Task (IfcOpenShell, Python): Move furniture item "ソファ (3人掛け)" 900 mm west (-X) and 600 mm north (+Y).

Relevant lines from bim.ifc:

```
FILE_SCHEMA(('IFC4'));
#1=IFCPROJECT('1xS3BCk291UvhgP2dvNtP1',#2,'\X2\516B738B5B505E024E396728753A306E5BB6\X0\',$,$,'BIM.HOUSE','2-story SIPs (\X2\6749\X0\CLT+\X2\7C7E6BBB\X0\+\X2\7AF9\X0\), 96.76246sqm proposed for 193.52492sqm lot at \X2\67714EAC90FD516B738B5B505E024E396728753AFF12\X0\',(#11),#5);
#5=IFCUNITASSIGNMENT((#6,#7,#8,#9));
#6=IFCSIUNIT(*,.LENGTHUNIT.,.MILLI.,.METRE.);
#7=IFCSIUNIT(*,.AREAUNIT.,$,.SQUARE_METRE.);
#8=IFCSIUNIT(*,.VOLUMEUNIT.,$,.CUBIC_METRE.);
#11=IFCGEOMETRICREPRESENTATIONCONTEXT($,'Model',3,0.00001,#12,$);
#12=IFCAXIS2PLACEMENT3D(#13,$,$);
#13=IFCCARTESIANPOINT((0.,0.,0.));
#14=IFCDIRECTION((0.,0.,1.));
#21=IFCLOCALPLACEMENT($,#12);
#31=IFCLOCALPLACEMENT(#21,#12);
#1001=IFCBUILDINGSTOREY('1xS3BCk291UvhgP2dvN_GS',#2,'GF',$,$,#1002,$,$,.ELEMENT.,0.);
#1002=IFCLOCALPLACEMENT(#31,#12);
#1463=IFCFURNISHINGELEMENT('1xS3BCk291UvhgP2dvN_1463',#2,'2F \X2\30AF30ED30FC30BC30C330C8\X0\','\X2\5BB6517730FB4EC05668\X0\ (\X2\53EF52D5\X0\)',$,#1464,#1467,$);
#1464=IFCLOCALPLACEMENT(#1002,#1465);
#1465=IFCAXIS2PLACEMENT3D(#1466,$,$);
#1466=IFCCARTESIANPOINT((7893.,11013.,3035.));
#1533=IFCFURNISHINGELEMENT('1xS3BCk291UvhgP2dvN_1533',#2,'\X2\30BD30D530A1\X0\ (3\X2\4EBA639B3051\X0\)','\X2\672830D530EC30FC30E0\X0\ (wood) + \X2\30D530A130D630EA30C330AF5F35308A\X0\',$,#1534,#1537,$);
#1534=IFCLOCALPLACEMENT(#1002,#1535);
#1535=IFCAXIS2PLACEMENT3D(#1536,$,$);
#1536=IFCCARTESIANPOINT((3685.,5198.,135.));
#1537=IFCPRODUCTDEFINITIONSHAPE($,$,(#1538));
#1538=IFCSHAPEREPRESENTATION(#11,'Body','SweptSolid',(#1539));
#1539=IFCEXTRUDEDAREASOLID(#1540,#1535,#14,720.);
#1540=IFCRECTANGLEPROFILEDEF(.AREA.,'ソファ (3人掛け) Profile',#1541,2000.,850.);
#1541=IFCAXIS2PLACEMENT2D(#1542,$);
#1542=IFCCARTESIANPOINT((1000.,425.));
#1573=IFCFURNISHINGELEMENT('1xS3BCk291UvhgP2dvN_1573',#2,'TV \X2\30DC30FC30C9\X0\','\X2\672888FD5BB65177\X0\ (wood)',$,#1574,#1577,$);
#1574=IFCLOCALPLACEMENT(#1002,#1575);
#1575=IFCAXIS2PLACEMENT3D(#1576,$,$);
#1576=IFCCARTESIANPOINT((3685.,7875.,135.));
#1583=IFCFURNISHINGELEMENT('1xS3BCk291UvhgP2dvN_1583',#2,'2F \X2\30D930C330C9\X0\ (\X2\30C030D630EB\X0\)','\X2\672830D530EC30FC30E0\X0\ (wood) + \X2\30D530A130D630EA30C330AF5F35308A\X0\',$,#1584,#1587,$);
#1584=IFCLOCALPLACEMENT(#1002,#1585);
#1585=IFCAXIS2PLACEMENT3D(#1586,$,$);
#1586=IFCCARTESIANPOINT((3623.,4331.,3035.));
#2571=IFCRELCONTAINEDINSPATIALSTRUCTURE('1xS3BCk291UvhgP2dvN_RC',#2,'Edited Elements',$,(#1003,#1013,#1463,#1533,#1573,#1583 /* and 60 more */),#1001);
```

```python
import ifcopenshell
import ifcopenshell.api.geometry
import ifcopenshell.util.placement

model = ifcopenshell.open("bim.ifc")

item = model.by_id(1533)
matrix = ifcopenshell.util.placement.get_local_placement(item.ObjectPlacement)
matrix[0, 3] -= 900.0
matrix[1, 3] += 600.0
ifcopenshell.api.geometry.edit_object_placement(model, product=item, matrix=matrix, is_si=False)

print(ifcopenshell.util.placement.get_local_placement(item.ObjectPlacement).round(3) + 0.0)

model.write("bim_rev.ifc")
```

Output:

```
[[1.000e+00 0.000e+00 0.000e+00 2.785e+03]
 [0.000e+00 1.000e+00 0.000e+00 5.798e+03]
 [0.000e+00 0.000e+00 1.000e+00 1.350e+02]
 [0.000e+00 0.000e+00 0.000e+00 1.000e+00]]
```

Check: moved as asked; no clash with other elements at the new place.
